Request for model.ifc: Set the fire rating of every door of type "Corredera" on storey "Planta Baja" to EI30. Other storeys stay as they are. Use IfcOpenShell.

First a look at what the model holds.

```python
import ifcopenshell
import ifcopenshell.util.element

model = ifcopenshell.open("model.ifc")
print(model.schema)
storey = next(s for s in model.by_type("IfcBuildingStorey") if s.Name == "Planta Baja")
doors = [e for e in ifcopenshell.util.element.get_decomposition(storey) if e.is_a("IfcDoor")]
seen = {}
for e in doors:
    element_type = ifcopenshell.util.element.get_type(e)
    key = (element_type.Name if element_type != e and element_type else None, ifcopenshell.util.element.get_pset(e, "Pset_DoorCommon", "FireRating"))
    seen[key] = seen.get(key, 0) + 1
for (name, value), count in sorted(seen.items(), key=str):
    print(count, "x", name, "|", value)
```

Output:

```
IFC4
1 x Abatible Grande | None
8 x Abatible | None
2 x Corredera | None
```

```python
import ifcopenshell
import ifcopenshell.api.pset
import ifcopenshell.util.element

model = ifcopenshell.open("model.ifc")

storey = next(s for s in model.by_type("IfcBuildingStorey") if s.Name == "Planta Baja")
doors = [e for e in ifcopenshell.util.element.get_decomposition(storey) if e.is_a("IfcDoor")]

count = 0
for e in doors:
    element_type = ifcopenshell.util.element.get_type(e)
    if element_type in (None, e) or element_type.Name != "Corredera":
        continue
    # add_pset returns the element's existing set when there is one.
    pset = ifcopenshell.api.pset.add_pset(model, product=e, name="Pset_DoorCommon")
    ifcopenshell.api.pset.edit_pset(model, pset=pset, properties={"FireRating": "EI30"})
    count += 1

print(count, "doors updated")

model.write("model_v2.ifc")
```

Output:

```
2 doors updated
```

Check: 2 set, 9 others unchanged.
